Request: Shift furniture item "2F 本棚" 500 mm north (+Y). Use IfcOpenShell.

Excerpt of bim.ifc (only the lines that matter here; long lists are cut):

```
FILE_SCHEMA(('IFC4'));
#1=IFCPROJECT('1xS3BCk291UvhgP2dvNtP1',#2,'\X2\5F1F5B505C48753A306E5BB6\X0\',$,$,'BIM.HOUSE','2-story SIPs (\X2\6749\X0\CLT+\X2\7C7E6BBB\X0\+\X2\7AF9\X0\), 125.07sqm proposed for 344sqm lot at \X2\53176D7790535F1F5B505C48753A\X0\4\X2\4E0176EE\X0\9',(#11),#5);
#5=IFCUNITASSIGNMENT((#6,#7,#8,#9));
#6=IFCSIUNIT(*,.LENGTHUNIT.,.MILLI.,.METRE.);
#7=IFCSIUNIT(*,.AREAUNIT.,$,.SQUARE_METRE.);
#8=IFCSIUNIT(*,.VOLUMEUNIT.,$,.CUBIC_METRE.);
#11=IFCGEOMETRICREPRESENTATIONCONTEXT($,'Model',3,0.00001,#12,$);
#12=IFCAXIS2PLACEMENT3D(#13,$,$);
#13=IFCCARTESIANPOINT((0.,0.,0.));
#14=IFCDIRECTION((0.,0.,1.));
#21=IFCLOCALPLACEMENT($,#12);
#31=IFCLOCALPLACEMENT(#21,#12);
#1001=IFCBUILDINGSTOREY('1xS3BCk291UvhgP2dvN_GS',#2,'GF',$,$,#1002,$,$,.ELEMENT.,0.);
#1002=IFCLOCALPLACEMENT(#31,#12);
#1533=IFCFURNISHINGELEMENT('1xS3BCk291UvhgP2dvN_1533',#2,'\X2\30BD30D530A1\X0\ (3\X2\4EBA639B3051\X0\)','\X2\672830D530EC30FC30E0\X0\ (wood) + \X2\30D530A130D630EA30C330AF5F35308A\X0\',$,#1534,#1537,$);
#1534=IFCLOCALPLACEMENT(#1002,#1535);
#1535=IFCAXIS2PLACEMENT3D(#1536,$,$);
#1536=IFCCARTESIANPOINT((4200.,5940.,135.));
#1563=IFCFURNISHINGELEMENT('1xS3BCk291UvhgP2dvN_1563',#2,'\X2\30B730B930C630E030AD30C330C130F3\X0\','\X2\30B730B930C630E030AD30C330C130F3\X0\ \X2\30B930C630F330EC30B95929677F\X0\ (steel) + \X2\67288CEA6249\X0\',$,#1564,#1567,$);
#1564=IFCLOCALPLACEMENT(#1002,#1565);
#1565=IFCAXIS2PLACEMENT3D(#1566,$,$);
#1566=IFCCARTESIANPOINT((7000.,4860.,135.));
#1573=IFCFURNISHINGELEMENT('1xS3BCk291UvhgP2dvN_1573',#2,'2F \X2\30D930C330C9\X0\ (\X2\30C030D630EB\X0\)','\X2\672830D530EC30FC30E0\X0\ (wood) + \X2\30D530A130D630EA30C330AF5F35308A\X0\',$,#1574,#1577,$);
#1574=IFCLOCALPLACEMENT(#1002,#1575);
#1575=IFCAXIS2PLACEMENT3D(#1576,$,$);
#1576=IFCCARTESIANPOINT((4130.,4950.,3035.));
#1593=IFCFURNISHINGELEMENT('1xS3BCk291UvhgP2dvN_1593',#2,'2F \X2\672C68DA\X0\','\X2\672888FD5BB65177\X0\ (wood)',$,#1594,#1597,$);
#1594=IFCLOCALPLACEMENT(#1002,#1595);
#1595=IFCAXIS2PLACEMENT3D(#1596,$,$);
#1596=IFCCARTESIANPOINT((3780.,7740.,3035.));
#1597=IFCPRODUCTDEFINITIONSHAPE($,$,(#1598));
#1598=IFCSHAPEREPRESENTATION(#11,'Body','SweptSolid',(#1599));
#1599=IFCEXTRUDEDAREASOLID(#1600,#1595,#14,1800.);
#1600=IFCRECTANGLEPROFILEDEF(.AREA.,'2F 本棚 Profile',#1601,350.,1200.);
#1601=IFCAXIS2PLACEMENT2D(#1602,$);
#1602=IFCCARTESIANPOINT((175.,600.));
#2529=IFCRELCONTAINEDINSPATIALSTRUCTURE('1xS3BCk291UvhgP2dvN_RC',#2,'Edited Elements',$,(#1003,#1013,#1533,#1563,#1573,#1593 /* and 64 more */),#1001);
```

```python
import ifcopenshell
import ifcopenshell.api.geometry
import ifcopenshell.util.placement

model = ifcopenshell.open("bim.ifc")

item = model.by_guid("1xS3BCk291UvhgP2dvN_1593")
matrix = ifcopenshell.util.placement.get_local_placement(item.ObjectPlacement)
matrix[1, 3] += 500.0
ifcopenshell.api.geometry.edit_object_placement(model, product=item, matrix=matrix, is_si=False)

print(ifcopenshell.util.placement.get_local_placement(item.ObjectPlacement).round(3) + 0.0)

model.write("bim-out.ifc")
```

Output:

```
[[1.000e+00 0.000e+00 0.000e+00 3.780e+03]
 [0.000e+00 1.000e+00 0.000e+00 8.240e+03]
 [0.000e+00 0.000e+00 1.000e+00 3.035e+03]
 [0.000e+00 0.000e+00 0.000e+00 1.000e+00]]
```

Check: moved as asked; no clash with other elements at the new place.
